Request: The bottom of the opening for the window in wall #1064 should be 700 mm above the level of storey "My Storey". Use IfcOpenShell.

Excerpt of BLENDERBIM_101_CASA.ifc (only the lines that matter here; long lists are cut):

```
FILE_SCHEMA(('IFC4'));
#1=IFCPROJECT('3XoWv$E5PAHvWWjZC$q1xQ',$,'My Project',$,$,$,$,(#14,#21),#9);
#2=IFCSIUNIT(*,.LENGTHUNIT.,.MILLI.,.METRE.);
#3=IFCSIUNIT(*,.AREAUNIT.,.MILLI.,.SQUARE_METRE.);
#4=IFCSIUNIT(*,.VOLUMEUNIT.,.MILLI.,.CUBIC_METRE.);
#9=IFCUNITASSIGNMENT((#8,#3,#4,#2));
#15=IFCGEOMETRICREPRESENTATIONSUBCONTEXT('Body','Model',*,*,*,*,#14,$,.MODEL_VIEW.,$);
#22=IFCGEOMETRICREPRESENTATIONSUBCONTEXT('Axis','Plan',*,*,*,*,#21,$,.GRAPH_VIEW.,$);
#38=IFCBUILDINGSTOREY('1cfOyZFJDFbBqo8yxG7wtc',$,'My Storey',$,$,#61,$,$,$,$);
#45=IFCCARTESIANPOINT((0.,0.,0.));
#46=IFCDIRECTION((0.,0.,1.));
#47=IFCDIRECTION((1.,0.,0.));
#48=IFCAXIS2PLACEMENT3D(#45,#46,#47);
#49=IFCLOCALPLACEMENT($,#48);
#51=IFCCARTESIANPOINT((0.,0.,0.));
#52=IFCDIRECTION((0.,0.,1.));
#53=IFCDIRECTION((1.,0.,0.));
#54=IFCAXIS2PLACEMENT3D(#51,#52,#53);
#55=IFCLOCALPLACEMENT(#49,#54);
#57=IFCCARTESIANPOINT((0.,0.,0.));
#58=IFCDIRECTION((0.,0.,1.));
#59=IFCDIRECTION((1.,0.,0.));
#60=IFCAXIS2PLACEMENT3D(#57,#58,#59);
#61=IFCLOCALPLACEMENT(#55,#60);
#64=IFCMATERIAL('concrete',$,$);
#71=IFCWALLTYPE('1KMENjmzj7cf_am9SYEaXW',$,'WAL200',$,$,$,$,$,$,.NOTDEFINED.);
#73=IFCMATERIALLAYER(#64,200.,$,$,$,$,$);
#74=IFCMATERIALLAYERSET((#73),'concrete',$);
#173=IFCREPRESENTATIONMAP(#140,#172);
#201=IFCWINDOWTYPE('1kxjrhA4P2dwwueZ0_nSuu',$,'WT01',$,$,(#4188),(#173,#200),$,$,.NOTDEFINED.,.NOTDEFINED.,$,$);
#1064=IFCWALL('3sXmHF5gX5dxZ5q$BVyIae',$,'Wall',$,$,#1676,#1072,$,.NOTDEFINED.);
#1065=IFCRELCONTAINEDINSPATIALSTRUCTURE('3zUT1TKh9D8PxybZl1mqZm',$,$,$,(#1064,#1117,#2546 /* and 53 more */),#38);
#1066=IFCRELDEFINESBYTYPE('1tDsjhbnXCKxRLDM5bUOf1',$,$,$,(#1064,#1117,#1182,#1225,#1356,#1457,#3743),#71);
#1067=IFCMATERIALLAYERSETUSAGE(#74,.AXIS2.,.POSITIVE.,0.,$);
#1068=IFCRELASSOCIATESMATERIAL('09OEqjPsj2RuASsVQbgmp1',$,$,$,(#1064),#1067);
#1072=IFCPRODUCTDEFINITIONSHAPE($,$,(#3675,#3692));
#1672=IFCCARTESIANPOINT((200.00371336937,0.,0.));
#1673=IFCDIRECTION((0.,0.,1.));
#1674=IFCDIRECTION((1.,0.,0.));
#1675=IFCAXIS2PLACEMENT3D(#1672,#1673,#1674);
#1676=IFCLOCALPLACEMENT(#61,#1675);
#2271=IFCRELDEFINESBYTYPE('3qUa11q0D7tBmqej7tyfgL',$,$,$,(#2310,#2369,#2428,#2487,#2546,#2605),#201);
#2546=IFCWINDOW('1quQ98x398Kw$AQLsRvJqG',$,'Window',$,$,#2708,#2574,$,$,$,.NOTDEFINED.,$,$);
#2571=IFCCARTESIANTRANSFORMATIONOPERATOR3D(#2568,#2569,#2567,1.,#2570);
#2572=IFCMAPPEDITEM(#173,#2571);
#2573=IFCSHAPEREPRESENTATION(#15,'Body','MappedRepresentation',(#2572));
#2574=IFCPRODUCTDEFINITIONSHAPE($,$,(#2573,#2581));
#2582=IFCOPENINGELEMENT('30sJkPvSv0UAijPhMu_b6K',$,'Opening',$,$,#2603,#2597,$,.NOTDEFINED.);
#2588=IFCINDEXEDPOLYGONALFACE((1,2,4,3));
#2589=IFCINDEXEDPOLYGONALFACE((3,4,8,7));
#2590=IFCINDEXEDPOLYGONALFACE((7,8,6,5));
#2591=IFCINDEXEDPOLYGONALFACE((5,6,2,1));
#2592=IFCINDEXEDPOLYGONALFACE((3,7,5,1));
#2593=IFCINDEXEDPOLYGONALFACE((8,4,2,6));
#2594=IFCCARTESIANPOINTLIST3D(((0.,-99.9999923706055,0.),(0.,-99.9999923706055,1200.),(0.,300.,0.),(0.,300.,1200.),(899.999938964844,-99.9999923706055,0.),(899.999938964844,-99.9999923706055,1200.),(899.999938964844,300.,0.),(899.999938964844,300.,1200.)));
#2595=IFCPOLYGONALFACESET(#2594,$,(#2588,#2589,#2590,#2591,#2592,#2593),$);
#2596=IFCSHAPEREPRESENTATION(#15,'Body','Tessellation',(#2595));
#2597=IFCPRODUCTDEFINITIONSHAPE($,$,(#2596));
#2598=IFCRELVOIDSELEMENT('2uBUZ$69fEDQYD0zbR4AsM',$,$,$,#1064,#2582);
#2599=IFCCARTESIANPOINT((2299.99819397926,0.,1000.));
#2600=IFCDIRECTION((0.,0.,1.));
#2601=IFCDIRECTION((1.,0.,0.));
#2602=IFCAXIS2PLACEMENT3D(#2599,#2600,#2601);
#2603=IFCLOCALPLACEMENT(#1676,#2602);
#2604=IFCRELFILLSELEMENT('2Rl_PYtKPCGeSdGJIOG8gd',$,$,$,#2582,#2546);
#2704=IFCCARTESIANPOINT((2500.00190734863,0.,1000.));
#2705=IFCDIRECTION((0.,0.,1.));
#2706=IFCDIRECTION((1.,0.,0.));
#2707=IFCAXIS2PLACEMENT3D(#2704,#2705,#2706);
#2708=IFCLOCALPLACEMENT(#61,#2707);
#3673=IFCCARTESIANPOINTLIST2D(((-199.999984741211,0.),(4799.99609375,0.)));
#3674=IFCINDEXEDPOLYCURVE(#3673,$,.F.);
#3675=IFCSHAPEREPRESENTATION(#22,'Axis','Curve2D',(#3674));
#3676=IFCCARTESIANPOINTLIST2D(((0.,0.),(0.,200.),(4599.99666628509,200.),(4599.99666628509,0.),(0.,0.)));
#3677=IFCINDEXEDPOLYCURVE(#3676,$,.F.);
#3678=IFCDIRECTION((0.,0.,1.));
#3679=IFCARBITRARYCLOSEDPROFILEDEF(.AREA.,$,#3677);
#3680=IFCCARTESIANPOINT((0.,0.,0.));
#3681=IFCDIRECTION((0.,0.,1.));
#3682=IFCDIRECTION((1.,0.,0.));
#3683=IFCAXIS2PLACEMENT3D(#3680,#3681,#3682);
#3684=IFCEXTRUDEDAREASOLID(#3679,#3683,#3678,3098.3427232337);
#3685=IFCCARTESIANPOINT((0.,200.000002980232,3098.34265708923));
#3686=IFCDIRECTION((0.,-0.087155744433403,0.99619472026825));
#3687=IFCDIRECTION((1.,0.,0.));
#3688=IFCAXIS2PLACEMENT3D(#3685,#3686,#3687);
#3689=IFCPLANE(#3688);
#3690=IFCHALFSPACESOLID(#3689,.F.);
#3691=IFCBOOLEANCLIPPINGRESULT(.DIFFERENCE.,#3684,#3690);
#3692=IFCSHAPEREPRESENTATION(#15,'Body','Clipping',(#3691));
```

```python
import numpy as np
import ifcopenshell
import ifcopenshell.api.geometry
import ifcopenshell.geom
import ifcopenshell.util.element
import ifcopenshell.util.placement
import ifcopenshell.util.shape
import ifcopenshell.util.unit

model = ifcopenshell.open("BLENDERBIM_101_CASA.ifc")
unit_scale = ifcopenshell.util.unit.calculate_unit_scale(model)

window = model.by_guid("1quQ98x398Kw$AQLsRvJqG")
opening = window.FillsVoids[0].RelatingOpeningElement
storey = ifcopenshell.util.element.get_container(window, ifc_class="IfcBuildingStorey")
level = ifcopenshell.util.placement.get_local_placement(storey.ObjectPlacement)[2, 3]

# The opening's origin need not be at the sill, so measure its lowest point.
shape = ifcopenshell.geom.create_shape(ifcopenshell.geom.settings(), opening)
bottom = ifcopenshell.util.shape.get_shape_bottom_elevation(shape, shape.geometry) / unit_scale
dz = level + 700.0 - bottom

shift = np.array([0.0, 0.0, dz])
# The window is not placed relative to its opening, so move both.
for product in (opening, window):
    matrix = ifcopenshell.util.placement.get_local_placement(product.ObjectPlacement)
    matrix[:3, 3] += shift
    ifcopenshell.api.geometry.edit_object_placement(model, product=product, matrix=matrix, is_si=False)

print(f"moved by {dz * unit_scale:+.3f} m")

model.write("BLENDERBIM_101_CASA_rev.ifc")
```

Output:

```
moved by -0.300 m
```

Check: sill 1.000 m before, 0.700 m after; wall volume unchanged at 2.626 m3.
